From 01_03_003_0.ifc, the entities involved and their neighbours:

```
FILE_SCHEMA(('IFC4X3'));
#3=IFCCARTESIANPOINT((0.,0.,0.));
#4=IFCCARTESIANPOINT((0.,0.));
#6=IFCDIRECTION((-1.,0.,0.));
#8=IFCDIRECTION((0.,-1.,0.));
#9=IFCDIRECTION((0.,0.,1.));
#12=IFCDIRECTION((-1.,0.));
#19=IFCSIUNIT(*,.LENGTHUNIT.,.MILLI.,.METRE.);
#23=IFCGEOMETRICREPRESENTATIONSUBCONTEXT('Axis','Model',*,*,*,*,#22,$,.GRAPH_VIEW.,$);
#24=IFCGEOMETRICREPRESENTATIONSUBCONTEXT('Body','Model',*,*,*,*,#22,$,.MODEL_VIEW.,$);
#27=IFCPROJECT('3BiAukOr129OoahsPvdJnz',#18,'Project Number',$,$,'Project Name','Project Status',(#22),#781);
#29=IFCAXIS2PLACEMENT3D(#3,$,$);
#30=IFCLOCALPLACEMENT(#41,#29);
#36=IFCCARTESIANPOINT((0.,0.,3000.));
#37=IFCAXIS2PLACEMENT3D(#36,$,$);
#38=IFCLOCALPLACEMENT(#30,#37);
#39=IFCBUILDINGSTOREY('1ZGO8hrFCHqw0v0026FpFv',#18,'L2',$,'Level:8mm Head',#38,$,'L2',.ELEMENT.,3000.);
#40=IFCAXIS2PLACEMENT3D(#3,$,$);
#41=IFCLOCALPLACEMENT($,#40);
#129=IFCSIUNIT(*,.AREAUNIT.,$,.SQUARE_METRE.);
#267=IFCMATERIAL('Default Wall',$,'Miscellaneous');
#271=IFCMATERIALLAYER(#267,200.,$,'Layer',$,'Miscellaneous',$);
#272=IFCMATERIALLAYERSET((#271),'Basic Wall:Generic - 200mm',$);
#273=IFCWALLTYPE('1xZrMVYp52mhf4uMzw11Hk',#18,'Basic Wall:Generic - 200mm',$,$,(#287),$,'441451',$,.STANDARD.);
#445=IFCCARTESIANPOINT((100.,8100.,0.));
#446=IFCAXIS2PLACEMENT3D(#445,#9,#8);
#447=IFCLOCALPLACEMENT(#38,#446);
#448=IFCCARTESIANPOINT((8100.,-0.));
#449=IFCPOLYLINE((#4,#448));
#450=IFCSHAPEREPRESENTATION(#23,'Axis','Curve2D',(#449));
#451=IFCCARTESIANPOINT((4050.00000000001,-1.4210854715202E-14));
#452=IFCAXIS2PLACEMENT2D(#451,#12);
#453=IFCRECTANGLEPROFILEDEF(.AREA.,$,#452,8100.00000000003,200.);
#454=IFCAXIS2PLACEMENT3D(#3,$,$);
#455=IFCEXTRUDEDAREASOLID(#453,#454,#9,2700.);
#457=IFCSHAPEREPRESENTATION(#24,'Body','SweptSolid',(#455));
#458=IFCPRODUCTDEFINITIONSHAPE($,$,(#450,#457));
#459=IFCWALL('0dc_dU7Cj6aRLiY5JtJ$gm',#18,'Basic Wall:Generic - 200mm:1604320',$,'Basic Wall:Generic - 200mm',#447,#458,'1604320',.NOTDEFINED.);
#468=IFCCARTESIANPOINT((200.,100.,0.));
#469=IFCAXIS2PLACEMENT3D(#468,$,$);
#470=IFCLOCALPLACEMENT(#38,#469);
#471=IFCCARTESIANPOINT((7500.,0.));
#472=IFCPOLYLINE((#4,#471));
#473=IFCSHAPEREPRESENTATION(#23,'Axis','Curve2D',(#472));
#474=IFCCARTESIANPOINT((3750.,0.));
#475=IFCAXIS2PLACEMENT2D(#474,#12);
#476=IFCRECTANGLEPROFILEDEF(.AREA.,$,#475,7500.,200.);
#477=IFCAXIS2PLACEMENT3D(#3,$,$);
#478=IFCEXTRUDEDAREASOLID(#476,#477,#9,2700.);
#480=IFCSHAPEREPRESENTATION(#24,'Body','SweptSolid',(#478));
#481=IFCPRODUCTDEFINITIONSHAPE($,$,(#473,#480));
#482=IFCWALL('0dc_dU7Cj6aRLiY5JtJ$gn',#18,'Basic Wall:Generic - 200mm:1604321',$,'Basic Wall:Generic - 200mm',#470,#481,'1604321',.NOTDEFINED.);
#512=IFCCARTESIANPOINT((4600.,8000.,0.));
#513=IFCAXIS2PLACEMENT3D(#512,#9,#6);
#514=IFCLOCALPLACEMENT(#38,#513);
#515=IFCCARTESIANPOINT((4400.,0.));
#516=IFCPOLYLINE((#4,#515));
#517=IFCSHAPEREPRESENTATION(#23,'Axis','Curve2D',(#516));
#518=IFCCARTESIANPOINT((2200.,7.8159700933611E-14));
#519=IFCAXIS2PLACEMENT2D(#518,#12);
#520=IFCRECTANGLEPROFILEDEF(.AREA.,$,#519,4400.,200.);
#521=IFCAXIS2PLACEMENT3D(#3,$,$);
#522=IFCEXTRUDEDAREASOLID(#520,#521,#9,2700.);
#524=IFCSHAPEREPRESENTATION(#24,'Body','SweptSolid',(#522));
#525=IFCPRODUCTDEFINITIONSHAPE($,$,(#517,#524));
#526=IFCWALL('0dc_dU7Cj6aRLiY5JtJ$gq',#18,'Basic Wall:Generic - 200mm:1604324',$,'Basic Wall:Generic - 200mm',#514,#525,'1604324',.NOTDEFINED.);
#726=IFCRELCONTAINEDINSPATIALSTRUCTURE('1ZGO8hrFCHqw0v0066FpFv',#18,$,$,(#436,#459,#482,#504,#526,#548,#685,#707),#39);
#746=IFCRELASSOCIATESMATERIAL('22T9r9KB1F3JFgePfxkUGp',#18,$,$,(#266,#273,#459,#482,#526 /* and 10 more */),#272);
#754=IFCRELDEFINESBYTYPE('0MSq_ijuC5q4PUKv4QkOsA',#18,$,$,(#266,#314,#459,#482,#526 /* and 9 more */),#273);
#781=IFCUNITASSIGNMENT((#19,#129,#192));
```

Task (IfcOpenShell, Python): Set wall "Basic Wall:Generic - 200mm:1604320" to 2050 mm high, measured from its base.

```python
import ifcopenshell
import ifcopenshell.geom
import ifcopenshell.util.representation
import ifcopenshell.util.shape
import ifcopenshell.util.unit

model = ifcopenshell.open("01_03_003_0.ifc")
unit_scale = ifcopenshell.util.unit.calculate_unit_scale(model)
settings = ifcopenshell.geom.settings()


def volume(element):
    """Net volume in cubic metres, openings subtracted."""
    shape = ifcopenshell.geom.create_shape(settings, element)
    return ifcopenshell.util.shape.get_volume(shape.geometry)


wall = model.by_id(459)
before = volume(wall)

body = ifcopenshell.util.representation.get_representation(wall, "Model", "Body")
solid = body.Items[0]
old_height = solid.Depth
solid.Depth = 2.05 / unit_scale
after = volume(wall)

print(f"height {old_height:g} -> {solid.Depth:g}, volume {before:.3f} -> {after:.3f} m3")

model.write("01_03_003_0_v2.ifc")
```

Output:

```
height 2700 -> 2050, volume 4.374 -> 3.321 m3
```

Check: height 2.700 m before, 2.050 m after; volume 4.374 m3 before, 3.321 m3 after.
